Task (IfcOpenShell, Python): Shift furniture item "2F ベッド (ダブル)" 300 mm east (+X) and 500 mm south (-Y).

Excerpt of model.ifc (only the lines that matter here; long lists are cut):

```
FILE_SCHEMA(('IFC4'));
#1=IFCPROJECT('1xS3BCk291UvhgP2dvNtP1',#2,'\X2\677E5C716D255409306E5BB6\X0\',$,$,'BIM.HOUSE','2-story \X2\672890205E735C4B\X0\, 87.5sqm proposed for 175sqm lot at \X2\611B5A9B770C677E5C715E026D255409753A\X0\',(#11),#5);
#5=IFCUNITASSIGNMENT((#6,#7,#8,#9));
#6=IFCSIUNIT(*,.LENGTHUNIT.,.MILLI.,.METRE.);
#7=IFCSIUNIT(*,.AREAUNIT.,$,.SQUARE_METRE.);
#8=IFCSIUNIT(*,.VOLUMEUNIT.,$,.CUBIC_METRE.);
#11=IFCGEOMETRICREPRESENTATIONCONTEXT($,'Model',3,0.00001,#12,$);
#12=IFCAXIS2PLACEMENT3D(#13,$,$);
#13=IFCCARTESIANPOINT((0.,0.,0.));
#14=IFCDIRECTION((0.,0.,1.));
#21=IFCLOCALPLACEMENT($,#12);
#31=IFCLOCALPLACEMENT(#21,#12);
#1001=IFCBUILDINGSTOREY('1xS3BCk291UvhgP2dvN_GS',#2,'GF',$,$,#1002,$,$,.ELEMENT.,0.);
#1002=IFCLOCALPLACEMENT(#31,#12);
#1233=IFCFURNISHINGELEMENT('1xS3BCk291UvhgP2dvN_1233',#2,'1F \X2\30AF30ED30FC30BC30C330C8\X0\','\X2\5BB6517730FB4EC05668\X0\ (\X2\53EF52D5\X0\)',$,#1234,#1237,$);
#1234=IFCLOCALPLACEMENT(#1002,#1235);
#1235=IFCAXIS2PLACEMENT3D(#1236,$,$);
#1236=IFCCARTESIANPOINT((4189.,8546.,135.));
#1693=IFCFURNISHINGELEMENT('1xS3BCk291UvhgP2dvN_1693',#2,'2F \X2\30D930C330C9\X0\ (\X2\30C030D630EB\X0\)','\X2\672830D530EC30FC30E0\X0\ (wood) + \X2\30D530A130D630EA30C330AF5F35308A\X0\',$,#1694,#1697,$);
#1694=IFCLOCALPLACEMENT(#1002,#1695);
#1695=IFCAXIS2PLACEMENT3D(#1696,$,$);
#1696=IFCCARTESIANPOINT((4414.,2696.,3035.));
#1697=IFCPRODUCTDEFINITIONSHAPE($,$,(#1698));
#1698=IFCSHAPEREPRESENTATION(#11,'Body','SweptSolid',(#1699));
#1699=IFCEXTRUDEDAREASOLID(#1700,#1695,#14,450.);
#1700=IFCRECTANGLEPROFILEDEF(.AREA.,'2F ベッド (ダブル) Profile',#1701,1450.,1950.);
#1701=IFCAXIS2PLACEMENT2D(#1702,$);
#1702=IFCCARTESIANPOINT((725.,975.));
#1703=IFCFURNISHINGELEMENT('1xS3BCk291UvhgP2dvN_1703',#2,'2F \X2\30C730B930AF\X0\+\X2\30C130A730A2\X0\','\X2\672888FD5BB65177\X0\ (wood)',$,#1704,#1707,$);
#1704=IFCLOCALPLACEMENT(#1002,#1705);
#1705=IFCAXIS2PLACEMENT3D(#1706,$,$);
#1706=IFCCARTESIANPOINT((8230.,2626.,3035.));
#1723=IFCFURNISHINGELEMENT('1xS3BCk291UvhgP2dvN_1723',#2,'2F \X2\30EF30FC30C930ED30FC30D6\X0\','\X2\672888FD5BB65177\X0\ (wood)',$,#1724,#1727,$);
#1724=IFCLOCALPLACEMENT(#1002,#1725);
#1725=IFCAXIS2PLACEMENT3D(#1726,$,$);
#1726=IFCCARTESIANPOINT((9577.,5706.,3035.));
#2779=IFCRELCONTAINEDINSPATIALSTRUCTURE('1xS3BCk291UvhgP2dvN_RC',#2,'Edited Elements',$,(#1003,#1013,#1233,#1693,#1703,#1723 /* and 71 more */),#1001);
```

```python
import ifcopenshell
import ifcopenshell.api.geometry
import ifcopenshell.util.placement
import ifcopenshell.util.unit

model = ifcopenshell.open("model.ifc")
unit_scale = ifcopenshell.util.unit.calculate_unit_scale(model)

item = model.by_guid("1xS3BCk291UvhgP2dvN_1693")
matrix = ifcopenshell.util.placement.get_local_placement(item.ObjectPlacement)
matrix[0, 3] += 0.3 / unit_scale
matrix[1, 3] -= 0.5 / unit_scale
ifcopenshell.api.geometry.edit_object_placement(model, product=item, matrix=matrix, is_si=False)

print(ifcopenshell.util.placement.get_local_placement(item.ObjectPlacement).round(3) + 0.0)

model.write("model_updated.ifc")
```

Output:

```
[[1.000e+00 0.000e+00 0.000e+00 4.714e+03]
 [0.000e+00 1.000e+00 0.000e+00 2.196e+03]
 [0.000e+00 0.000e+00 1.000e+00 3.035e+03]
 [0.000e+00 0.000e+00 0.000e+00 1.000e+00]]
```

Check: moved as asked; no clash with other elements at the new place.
